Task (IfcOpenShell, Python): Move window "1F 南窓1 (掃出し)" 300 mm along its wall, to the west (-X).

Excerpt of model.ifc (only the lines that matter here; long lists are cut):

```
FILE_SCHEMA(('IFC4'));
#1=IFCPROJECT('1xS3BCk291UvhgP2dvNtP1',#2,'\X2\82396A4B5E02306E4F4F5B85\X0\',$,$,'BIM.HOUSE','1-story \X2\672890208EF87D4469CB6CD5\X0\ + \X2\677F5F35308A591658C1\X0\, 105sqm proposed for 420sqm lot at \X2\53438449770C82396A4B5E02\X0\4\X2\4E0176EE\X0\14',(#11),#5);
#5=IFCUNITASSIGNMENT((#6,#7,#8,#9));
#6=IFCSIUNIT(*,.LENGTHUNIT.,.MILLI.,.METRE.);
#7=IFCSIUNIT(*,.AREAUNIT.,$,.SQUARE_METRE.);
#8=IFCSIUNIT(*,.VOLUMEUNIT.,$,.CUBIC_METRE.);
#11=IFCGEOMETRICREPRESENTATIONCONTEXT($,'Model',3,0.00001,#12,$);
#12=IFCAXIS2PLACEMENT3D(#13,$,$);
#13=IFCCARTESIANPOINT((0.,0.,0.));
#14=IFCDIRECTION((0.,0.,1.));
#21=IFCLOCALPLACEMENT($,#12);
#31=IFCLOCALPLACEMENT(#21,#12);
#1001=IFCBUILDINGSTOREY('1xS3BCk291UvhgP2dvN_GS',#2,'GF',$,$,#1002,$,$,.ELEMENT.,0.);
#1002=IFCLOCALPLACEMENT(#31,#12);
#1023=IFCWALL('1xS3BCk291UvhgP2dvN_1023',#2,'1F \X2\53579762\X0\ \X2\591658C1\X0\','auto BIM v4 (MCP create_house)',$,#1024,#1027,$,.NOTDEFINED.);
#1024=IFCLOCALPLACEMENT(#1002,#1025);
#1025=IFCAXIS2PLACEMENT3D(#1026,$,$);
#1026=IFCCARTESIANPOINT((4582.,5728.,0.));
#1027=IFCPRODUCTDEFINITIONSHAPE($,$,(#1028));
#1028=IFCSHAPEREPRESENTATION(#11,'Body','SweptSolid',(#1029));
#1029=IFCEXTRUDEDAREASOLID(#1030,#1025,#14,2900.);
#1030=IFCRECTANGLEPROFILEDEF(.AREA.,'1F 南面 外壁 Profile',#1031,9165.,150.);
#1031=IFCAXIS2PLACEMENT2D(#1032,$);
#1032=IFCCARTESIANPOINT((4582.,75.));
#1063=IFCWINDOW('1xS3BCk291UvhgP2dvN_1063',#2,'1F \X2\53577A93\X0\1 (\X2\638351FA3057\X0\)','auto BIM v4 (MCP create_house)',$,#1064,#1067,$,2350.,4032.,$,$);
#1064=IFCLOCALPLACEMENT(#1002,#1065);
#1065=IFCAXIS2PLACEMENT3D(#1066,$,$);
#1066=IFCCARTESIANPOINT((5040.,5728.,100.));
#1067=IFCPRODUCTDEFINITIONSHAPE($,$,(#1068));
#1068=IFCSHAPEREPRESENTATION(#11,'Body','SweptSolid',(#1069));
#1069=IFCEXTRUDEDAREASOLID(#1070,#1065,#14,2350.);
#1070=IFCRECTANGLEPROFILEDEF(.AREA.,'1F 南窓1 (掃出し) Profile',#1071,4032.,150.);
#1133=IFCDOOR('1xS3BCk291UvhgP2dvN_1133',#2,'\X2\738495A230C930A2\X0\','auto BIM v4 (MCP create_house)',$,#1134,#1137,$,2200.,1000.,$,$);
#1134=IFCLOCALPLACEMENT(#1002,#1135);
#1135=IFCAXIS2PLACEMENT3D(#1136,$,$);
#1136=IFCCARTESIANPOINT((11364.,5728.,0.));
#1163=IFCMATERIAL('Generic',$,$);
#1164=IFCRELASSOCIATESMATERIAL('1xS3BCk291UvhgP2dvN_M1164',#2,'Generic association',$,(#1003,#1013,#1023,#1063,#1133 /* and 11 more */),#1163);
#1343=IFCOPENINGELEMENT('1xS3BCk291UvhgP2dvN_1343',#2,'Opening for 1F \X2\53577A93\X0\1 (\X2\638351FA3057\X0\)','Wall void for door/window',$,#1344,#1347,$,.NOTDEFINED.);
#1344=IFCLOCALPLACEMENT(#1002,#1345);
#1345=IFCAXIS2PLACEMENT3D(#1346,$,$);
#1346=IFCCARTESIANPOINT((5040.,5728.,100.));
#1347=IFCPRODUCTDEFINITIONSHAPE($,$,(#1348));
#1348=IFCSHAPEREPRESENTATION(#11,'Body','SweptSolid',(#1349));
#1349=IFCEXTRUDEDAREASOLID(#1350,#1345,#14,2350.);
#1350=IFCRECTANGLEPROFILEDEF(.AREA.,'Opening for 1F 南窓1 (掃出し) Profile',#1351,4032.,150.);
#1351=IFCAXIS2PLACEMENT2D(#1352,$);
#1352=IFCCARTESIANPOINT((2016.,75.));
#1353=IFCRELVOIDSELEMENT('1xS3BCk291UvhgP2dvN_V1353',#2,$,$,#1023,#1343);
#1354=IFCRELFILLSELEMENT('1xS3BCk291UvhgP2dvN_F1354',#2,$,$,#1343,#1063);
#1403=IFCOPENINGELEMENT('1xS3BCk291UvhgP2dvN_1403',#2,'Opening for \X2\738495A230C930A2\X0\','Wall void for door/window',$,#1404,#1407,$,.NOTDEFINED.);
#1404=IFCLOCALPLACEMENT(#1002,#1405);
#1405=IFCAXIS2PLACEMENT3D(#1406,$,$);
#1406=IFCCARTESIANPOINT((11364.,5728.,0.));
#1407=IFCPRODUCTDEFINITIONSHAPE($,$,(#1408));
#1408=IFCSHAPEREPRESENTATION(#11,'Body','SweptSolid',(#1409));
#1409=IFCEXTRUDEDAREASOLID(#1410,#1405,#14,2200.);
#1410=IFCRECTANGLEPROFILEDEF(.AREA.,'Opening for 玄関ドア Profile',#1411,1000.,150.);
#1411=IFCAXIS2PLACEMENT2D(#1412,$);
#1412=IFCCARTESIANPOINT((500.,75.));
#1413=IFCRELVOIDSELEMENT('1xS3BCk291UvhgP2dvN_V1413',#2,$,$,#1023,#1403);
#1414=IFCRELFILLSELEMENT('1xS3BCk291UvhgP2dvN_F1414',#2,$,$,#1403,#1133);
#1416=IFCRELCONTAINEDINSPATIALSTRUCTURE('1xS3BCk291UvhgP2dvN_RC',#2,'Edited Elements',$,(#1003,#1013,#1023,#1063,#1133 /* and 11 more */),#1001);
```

```python
import ifcopenshell
import ifcopenshell.api.geometry
import ifcopenshell.util.placement
import ifcopenshell.util.unit

model = ifcopenshell.open("model.ifc")
unit_scale = ifcopenshell.util.unit.calculate_unit_scale(model)

window = model.by_id(1063)
opening = window.FillsVoids[0].RelatingOpeningElement
wall = opening.VoidsElements[0].RelatingBuildingElement

wall_matrix = ifcopenshell.util.placement.get_local_placement(wall.ObjectPlacement)
shift = wall_matrix[:3, 0] * -0.3 / unit_scale
before = ifcopenshell.util.placement.get_local_placement(window.ObjectPlacement)[:3, 3].copy()

# The window is not placed relative to its opening, so move both.
for product in (opening, window):
    matrix = ifcopenshell.util.placement.get_local_placement(product.ObjectPlacement)
    matrix[:3, 3] += shift
    ifcopenshell.api.geometry.edit_object_placement(model, product=product, matrix=matrix, is_si=False)

after = ifcopenshell.util.placement.get_local_placement(window.ObjectPlacement)[:3, 3]
print("window moved by", (after - before).round(3) + 0.0)

model.write("model_rev.ifc")
```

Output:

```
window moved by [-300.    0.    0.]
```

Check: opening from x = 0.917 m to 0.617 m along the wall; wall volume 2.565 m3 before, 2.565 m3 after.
